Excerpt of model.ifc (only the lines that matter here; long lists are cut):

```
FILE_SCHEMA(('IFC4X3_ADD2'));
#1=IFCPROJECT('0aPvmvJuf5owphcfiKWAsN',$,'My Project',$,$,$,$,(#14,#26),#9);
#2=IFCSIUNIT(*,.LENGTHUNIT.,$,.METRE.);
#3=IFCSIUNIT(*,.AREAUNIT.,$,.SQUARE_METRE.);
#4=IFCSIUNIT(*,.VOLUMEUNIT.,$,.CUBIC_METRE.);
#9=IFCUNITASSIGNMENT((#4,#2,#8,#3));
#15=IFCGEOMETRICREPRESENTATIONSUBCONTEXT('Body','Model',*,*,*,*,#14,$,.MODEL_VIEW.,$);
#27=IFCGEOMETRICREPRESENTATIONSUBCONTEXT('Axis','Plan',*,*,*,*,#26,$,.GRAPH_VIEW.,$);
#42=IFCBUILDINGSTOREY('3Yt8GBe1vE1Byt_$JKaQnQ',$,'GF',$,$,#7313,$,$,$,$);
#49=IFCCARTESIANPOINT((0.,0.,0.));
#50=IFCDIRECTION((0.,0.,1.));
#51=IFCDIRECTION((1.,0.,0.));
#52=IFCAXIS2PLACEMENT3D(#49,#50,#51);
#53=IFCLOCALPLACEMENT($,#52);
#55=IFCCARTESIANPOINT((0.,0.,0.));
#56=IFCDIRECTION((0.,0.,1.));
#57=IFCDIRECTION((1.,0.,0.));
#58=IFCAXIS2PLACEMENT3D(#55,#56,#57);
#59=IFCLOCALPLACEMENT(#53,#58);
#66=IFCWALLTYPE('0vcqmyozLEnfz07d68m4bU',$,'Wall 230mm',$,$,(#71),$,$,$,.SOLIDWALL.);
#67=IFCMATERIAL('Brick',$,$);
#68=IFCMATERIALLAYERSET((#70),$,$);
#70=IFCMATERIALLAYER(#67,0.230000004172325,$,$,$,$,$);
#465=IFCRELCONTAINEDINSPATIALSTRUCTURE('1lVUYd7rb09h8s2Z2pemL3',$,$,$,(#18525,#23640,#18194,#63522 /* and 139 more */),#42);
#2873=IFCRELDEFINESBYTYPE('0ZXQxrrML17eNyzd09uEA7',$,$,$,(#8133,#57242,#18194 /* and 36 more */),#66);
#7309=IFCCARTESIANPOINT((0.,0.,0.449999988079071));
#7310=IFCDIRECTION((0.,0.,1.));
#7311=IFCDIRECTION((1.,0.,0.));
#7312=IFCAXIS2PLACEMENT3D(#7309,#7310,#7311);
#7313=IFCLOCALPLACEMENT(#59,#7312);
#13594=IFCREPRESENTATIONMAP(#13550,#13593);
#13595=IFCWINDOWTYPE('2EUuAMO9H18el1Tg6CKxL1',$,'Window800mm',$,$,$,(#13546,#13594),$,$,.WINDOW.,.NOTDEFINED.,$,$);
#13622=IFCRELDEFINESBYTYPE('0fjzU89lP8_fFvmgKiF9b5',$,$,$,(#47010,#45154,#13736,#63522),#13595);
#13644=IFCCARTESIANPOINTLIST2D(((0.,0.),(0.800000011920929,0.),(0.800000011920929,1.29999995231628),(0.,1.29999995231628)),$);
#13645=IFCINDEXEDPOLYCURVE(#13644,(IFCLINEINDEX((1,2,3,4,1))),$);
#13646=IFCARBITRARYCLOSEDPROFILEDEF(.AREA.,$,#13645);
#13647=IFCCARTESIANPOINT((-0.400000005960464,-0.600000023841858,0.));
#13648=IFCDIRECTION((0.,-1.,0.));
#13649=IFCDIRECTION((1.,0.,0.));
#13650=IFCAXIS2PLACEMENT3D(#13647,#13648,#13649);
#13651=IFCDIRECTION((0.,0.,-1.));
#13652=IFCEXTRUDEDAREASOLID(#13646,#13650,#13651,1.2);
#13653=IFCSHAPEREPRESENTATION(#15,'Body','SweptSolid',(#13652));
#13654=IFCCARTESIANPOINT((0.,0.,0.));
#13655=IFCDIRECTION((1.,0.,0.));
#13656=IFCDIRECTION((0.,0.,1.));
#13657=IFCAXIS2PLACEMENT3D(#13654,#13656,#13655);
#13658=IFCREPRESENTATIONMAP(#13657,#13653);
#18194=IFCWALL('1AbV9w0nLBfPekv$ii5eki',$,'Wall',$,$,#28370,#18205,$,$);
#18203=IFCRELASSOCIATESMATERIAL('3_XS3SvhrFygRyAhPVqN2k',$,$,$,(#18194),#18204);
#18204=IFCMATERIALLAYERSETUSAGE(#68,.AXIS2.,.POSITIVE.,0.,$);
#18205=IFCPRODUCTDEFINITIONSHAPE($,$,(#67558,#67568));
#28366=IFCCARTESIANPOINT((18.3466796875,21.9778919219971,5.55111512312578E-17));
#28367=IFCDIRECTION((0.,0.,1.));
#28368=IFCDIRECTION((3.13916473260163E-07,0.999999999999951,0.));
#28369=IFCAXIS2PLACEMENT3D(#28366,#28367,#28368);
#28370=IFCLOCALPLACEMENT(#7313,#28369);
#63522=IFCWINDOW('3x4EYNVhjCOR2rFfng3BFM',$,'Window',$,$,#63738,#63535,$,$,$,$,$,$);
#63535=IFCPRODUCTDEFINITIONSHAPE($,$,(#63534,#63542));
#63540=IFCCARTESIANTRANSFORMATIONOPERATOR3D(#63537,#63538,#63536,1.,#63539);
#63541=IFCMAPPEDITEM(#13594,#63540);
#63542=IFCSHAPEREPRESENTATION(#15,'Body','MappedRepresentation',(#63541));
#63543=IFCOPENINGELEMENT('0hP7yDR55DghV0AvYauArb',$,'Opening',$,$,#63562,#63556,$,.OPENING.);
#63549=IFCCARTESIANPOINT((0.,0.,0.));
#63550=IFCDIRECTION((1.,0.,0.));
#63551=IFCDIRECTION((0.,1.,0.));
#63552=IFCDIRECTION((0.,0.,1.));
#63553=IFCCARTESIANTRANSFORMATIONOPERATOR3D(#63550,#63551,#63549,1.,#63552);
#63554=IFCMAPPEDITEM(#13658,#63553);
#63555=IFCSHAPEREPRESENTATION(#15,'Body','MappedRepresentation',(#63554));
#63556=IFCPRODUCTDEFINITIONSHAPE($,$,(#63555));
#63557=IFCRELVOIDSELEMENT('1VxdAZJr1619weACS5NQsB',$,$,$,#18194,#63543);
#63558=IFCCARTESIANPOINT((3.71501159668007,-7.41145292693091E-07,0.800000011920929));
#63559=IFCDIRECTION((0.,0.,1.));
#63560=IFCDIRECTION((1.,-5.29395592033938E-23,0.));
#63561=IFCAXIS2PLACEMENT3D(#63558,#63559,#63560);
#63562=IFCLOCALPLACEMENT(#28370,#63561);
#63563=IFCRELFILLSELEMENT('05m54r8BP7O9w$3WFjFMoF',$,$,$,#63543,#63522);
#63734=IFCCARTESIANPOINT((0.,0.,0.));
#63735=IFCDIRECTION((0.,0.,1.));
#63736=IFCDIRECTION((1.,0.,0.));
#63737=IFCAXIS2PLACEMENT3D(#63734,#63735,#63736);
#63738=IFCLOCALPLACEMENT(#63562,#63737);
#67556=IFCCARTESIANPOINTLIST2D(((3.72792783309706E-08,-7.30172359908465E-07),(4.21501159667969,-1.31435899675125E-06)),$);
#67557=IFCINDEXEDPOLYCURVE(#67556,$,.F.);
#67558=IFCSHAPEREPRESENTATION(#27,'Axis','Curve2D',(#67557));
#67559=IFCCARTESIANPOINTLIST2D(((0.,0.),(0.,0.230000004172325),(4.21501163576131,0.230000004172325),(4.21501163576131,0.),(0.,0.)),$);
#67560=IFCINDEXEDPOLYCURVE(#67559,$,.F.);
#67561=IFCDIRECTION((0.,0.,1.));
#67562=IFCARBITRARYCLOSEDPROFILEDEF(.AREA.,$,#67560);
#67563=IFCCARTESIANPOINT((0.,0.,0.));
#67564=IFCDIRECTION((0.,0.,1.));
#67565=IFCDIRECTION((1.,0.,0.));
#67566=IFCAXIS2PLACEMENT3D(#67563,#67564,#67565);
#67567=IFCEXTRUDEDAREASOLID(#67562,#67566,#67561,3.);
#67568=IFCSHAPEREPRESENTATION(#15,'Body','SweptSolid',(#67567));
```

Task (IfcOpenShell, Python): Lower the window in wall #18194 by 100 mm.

```python
import numpy as np
import ifcopenshell
import ifcopenshell.api.geometry
import ifcopenshell.util.placement
import ifcopenshell.util.unit

model = ifcopenshell.open("model.ifc")
unit_scale = ifcopenshell.util.unit.calculate_unit_scale(model)

window = model.by_guid("3x4EYNVhjCOR2rFfng3BFM")
opening = window.FillsVoids[0].RelatingOpeningElement
dz = -0.1

shift = np.array([0.0, 0.0, dz])
# The window is placed relative to its opening, so it follows when the opening moves.
matrix = ifcopenshell.util.placement.get_local_placement(opening.ObjectPlacement)
matrix[:3, 3] += shift
ifcopenshell.api.geometry.edit_object_placement(
    model, product=opening, matrix=matrix, is_si=False, should_transform_children=True
)

print(f"moved by {dz * unit_scale:+.3f} m")

model.write("model_v2.ifc")
```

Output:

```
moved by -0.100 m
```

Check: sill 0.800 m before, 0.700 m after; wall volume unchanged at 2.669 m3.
